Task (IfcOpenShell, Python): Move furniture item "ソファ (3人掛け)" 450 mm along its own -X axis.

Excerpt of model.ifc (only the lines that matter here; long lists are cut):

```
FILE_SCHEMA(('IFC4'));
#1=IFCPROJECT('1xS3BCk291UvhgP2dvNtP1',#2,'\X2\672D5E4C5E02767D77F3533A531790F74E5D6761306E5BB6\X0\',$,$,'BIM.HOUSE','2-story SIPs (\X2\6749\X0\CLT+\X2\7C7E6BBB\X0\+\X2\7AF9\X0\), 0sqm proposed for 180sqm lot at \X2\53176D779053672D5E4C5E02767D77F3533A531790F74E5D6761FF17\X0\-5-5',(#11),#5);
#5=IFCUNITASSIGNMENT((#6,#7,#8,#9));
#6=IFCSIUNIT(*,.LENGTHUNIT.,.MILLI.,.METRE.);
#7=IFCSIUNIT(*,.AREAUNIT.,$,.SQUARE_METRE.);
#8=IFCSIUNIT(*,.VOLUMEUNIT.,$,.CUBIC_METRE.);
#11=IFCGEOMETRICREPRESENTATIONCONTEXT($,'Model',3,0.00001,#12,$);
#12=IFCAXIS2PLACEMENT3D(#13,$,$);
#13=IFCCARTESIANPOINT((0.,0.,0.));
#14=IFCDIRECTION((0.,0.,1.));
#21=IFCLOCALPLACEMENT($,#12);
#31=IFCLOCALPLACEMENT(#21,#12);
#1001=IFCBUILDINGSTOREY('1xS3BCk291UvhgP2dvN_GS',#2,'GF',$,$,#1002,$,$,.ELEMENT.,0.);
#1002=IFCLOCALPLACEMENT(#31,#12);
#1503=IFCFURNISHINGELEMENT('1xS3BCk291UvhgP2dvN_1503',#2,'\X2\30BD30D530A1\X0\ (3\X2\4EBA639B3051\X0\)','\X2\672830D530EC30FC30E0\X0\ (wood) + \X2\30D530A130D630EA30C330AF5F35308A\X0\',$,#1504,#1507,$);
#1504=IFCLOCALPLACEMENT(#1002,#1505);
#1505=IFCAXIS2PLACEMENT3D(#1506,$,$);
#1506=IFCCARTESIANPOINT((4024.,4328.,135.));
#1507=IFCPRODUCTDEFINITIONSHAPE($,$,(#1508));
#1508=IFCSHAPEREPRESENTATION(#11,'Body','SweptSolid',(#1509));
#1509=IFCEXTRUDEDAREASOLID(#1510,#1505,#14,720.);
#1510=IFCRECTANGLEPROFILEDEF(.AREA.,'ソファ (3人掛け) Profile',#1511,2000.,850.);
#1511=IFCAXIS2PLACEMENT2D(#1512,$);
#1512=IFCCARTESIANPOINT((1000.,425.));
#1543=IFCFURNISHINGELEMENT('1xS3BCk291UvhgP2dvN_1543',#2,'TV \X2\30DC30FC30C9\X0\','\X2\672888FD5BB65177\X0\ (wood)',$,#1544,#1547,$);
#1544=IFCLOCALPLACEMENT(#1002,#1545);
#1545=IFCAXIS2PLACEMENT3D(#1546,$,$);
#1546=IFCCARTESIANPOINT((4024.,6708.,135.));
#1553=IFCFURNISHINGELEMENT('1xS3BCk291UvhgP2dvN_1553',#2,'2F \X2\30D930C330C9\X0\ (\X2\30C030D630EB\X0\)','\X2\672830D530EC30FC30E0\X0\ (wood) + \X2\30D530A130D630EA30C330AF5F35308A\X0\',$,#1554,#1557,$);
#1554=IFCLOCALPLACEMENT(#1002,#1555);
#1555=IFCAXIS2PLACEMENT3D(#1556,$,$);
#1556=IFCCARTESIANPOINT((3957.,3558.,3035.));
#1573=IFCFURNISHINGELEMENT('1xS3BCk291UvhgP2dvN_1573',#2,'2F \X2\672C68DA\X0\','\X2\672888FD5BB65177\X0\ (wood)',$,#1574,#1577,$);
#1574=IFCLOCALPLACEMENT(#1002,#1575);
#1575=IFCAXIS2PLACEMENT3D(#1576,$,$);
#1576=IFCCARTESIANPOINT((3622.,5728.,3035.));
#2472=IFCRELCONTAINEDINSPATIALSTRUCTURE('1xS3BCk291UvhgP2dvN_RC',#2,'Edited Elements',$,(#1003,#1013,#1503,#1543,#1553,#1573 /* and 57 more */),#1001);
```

```python
import ifcopenshell
import ifcopenshell.api.geometry
import ifcopenshell.util.placement

model = ifcopenshell.open("model.ifc")

item = model.by_guid("1xS3BCk291UvhgP2dvN_1503")
matrix = ifcopenshell.util.placement.get_local_placement(item.ObjectPlacement)
matrix[:3, 3] -= matrix[:3, 0] * 450.0
ifcopenshell.api.geometry.edit_object_placement(model, product=item, matrix=matrix, is_si=False)

print(ifcopenshell.util.placement.get_local_placement(item.ObjectPlacement).round(3) + 0.0)

model.write("model_rev.ifc")
```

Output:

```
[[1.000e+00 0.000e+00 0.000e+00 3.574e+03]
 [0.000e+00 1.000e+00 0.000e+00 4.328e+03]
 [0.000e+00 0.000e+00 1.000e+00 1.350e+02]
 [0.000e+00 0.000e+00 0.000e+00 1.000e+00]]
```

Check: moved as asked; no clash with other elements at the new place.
